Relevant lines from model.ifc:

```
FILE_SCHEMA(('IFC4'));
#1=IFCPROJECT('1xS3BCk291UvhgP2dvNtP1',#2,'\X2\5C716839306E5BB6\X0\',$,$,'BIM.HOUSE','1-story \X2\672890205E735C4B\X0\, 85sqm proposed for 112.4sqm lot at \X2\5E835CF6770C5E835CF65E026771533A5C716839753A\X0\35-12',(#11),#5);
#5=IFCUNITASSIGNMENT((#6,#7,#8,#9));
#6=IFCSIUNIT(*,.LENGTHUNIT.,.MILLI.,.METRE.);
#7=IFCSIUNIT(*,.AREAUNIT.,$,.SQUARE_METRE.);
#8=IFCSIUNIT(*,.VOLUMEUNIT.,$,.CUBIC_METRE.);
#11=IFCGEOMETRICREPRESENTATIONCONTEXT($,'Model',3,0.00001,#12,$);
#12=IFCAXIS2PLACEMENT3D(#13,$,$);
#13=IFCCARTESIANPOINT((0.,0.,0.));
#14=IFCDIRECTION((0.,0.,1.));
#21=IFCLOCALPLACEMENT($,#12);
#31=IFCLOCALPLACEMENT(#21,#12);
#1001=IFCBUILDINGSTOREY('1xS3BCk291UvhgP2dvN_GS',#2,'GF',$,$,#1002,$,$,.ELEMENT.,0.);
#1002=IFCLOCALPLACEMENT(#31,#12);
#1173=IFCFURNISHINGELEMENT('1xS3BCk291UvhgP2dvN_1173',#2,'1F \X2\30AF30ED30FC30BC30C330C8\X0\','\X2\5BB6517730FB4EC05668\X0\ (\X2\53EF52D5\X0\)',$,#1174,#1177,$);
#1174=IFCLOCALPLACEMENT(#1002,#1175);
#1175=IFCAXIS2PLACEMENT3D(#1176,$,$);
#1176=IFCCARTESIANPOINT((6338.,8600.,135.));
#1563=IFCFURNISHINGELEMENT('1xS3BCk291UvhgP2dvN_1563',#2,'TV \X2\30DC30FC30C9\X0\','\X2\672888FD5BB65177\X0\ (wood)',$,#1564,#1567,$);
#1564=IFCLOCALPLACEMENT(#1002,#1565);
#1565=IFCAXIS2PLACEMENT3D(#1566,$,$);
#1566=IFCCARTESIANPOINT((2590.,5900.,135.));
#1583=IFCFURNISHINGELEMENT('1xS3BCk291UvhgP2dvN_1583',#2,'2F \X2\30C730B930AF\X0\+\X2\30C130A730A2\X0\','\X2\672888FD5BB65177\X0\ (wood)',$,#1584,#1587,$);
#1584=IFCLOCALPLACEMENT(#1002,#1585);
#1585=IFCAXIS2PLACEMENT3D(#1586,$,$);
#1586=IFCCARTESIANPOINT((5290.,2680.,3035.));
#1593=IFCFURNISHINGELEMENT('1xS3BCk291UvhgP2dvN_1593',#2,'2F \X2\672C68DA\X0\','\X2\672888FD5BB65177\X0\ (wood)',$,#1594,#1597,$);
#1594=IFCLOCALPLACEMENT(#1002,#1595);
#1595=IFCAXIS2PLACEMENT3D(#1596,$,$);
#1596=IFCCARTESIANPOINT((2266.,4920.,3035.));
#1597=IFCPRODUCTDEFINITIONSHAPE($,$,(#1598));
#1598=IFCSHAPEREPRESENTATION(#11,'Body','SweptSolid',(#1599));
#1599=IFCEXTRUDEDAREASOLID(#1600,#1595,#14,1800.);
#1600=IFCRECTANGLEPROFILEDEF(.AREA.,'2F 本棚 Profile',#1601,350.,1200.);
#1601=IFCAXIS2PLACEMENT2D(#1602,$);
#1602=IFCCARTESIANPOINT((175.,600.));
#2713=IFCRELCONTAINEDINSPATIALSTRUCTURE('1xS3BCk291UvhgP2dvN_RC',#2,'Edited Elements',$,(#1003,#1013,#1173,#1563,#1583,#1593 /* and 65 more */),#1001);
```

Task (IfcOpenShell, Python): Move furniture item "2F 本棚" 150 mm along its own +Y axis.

```python
import ifcopenshell
import ifcopenshell.api.geometry
import ifcopenshell.util.placement

model = ifcopenshell.open("model.ifc")

item = model.by_id(1593)
matrix = ifcopenshell.util.placement.get_local_placement(item.ObjectPlacement)
matrix[:3, 3] += matrix[:3, 1] * 150.0
ifcopenshell.api.geometry.edit_object_placement(model, product=item, matrix=matrix, is_si=False)

print(ifcopenshell.util.placement.get_local_placement(item.ObjectPlacement).round(3) + 0.0)

model.write("model_rev.ifc")
```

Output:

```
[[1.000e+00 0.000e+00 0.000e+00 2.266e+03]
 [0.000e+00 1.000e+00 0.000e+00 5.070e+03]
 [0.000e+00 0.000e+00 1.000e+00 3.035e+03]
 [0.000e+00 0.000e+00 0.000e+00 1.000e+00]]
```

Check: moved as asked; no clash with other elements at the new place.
